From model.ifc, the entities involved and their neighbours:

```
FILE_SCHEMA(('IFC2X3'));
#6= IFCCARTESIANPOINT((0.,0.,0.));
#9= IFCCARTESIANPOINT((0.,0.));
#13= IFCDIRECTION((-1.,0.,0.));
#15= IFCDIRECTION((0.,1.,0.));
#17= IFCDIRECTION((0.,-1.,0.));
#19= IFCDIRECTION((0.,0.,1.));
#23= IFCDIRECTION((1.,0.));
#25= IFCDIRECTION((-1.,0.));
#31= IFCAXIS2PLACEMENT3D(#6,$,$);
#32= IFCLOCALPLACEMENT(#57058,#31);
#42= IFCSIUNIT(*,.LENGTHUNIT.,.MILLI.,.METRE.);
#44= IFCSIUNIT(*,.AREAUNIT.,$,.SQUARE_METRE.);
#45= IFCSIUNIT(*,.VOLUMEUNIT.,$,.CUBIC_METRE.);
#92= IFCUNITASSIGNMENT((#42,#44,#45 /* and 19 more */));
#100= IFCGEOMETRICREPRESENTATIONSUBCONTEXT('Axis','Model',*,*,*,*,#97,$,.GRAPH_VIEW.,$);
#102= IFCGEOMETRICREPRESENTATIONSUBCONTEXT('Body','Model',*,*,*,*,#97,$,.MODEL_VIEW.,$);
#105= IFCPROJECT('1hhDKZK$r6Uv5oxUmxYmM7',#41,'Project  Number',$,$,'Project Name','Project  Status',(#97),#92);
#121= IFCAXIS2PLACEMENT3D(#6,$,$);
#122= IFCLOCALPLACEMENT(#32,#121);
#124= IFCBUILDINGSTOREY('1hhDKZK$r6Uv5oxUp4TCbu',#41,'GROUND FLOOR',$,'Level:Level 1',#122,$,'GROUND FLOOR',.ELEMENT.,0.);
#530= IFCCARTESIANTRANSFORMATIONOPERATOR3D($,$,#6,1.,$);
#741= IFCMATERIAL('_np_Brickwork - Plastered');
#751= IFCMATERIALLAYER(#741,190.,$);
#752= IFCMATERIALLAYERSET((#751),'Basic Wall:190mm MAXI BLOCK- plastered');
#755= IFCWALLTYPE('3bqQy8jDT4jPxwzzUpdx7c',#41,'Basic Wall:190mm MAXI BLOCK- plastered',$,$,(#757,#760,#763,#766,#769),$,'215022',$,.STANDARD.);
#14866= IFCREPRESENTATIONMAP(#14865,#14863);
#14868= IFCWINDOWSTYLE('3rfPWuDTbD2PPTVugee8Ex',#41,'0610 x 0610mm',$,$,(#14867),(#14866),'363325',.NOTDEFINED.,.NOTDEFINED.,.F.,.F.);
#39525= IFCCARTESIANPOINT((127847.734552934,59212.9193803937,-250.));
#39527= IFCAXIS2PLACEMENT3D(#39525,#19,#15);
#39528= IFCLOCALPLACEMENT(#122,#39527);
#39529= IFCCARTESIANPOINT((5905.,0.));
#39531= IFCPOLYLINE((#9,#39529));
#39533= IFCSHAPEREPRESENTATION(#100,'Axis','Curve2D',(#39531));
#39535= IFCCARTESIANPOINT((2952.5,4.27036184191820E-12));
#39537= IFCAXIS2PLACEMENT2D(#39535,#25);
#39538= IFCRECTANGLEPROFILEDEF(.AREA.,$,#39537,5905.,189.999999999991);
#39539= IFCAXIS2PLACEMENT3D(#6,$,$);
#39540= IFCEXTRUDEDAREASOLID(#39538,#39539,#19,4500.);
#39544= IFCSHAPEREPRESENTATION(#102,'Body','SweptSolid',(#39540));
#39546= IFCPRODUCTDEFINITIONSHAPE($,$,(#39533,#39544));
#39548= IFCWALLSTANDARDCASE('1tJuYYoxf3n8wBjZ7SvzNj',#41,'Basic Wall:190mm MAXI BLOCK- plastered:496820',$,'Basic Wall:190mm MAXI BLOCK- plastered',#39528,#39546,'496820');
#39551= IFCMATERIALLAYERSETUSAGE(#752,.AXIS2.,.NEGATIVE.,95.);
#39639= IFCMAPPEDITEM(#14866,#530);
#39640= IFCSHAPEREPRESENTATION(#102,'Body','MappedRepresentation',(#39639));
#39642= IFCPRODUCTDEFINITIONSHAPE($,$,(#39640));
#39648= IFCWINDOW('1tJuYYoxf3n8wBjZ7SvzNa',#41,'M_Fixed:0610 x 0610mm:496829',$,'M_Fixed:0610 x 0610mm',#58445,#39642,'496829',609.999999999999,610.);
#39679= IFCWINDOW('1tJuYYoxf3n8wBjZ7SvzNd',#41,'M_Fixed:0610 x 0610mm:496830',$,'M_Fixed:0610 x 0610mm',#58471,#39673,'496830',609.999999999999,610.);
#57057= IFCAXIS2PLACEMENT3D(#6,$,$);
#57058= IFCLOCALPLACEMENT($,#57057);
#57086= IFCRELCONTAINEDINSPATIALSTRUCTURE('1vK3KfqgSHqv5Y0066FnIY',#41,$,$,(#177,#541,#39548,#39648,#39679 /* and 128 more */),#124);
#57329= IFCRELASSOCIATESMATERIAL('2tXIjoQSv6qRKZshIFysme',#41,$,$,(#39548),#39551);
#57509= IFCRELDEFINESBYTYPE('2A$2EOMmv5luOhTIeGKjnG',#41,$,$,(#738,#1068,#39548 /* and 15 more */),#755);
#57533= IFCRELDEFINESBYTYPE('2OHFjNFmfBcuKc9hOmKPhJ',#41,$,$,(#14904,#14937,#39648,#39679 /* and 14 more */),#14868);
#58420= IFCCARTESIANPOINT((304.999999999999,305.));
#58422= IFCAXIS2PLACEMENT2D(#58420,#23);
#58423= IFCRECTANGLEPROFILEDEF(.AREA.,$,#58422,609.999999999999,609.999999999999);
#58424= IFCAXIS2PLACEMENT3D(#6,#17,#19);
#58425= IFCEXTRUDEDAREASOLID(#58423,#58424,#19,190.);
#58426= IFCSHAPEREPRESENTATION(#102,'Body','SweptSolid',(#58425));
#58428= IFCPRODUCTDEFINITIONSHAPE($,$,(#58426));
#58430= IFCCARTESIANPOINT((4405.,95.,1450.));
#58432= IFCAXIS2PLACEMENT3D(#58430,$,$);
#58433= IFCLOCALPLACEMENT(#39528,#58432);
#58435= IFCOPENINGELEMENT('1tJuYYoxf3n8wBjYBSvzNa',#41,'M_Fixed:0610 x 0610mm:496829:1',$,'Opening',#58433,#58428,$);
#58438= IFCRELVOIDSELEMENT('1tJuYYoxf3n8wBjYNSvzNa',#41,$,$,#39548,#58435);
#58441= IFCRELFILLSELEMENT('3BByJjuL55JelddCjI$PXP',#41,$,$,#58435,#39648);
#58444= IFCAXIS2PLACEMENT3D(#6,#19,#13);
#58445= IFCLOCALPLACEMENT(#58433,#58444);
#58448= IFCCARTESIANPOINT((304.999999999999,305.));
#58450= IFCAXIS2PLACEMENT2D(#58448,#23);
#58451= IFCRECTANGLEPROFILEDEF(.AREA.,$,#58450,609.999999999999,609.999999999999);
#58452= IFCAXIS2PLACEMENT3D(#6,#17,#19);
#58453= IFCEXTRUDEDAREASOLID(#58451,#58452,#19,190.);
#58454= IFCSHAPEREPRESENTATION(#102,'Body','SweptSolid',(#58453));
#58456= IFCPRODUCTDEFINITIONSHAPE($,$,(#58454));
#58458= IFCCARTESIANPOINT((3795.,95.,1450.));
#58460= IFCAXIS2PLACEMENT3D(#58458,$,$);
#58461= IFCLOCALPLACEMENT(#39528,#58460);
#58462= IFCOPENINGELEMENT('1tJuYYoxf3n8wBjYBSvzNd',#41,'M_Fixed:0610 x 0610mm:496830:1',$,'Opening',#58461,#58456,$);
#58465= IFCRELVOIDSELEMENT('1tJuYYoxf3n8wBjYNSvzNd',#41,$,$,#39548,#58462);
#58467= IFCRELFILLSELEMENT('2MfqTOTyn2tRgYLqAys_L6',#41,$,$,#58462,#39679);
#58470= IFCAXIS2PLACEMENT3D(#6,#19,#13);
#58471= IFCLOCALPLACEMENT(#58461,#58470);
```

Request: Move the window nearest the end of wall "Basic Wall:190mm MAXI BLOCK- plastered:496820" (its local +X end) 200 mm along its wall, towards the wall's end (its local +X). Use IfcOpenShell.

```python
import ifcopenshell
import ifcopenshell.api.geometry
import ifcopenshell.util.placement
import ifcopenshell.util.unit

model = ifcopenshell.open("model.ifc")
unit_scale = ifcopenshell.util.unit.calculate_unit_scale(model)

window = model.by_guid("1tJuYYoxf3n8wBjZ7SvzNa")
opening = window.FillsVoids[0].RelatingOpeningElement
wall = opening.VoidsElements[0].RelatingBuildingElement

wall_matrix = ifcopenshell.util.placement.get_local_placement(wall.ObjectPlacement)
shift = wall_matrix[:3, 0] * 0.2 / unit_scale
before = ifcopenshell.util.placement.get_local_placement(window.ObjectPlacement)[:3, 3].copy()

# The window is placed relative to its opening, so it follows when the opening moves.
matrix = ifcopenshell.util.placement.get_local_placement(opening.ObjectPlacement)
matrix[:3, 3] += shift
ifcopenshell.api.geometry.edit_object_placement(
    model, product=opening, matrix=matrix, is_si=False, should_transform_children=True
)

after = ifcopenshell.util.placement.get_local_placement(window.ObjectPlacement)[:3, 3]
print("window moved by", (after - before).round(3) + 0.0)

model.write("model-out.ifc")
```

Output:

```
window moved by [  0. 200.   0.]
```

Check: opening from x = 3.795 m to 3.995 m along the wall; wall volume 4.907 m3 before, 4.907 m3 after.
